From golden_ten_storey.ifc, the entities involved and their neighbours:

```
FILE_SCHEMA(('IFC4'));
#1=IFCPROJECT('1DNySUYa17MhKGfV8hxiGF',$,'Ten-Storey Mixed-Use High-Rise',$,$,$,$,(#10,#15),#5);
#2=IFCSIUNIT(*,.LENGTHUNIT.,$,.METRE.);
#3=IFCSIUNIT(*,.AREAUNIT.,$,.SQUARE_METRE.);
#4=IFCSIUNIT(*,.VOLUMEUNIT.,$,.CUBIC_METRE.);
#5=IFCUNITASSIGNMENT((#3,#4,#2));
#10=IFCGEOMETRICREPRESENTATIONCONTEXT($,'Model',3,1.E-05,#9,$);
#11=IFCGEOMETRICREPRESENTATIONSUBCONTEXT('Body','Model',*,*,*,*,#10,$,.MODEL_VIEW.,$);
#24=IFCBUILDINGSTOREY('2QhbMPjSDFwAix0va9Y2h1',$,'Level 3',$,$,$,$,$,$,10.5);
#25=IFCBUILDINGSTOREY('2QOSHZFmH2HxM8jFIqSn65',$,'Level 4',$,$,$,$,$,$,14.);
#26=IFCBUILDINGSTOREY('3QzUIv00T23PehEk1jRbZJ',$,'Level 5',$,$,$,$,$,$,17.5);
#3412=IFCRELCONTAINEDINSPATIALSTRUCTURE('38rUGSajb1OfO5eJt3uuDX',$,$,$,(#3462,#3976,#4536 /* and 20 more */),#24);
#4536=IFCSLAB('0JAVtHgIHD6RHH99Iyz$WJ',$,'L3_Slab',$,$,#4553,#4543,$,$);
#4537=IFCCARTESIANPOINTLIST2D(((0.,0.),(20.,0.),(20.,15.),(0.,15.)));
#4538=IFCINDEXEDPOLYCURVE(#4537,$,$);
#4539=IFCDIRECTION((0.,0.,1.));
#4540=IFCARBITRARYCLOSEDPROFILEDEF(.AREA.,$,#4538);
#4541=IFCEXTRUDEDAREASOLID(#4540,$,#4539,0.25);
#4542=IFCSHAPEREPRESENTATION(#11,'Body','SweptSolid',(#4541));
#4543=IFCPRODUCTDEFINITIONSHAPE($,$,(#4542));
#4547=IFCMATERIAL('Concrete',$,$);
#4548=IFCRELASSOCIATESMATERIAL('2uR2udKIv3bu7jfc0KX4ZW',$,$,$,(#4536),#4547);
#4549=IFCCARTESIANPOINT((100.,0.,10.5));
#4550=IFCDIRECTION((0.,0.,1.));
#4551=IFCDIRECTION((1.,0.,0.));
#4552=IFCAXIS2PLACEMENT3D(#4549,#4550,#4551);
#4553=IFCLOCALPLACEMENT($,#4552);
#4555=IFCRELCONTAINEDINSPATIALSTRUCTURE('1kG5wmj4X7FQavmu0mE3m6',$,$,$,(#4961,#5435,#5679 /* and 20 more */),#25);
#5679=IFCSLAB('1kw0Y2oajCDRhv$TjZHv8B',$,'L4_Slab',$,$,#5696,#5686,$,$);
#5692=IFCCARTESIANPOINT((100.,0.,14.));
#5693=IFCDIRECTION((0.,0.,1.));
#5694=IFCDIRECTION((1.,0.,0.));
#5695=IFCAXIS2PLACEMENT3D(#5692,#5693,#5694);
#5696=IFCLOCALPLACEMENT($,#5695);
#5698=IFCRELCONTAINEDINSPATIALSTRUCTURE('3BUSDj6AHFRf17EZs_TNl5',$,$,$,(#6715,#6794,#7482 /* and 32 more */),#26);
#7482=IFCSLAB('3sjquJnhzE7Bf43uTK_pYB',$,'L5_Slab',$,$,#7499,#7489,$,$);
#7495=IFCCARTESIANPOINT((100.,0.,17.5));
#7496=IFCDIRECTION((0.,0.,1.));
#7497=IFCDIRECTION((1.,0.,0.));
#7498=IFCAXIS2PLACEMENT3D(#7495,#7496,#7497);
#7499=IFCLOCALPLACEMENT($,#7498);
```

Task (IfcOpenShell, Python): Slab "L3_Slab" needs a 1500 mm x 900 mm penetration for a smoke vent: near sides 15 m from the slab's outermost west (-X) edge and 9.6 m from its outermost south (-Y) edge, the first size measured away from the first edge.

```python
import numpy as np
import ifcopenshell
import ifcopenshell.api.feature
import ifcopenshell.api.geometry
import ifcopenshell.api.root
import ifcopenshell.geom
import ifcopenshell.util.placement
import ifcopenshell.util.representation
import ifcopenshell.util.shape
import ifcopenshell.util.unit

model = ifcopenshell.open("golden_ten_storey.ifc")
unit_scale = ifcopenshell.util.unit.calculate_unit_scale(model)
settings = ifcopenshell.geom.settings()


def volume(element):
    """Net volume in cubic metres, openings subtracted."""
    shape = ifcopenshell.geom.create_shape(settings, element)
    return ifcopenshell.util.shape.get_volume(shape.geometry)


slab = model.by_guid("0JAVtHgIHD6RHH99Iyz$WJ")
before = volume(slab)

# Extent in the slab's own axes, in metres. The edges named are its -X and -Y sides.
slab_shape = ifcopenshell.geom.create_shape(settings, slab)
vertices = ifcopenshell.util.shape.get_vertices(slab_shape.geometry)
x_min, y_min, bottom = vertices.min(axis=0)
top = vertices[:, 2].max()

opening = ifcopenshell.api.root.create_entity(model, ifc_class="IfcOpeningElement", name="Smoke vent opening", predefined_type="OPENING")
context = ifcopenshell.util.representation.get_context(model, "Model", "Body", "MODEL_VIEW")
width, depth = 1.5, 0.9
outline = [(0.0, 0.0), (width, 0.0), (width, depth), (0.0, depth), (0.0, 0.0)]
# Overshoot both faces by 50 mm so the cut is clean.
shape = ifcopenshell.api.geometry.add_slab_representation(
    model, context=context, depth=top - bottom + 0.1, polyline=outline
)
ifcopenshell.api.geometry.assign_representation(model, product=opening, representation=shape)

matrix = ifcopenshell.util.placement.get_local_placement(slab.ObjectPlacement)
matrix[:, 3] = matrix @ np.append(np.array([x_min + 15, y_min + 9.6, bottom - 0.05]) / unit_scale, 1.0)
ifcopenshell.api.geometry.edit_object_placement(model, product=opening, matrix=matrix, is_si=False)
ifcopenshell.api.feature.add_feature(model, feature=opening, element=slab)

after = volume(slab)

print(f"slab volume {before:.3f} -> {after:.3f} m3")

model.write("golden_ten_storey_updated.ifc")
```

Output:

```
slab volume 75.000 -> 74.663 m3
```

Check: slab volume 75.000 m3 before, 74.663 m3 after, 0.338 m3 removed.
